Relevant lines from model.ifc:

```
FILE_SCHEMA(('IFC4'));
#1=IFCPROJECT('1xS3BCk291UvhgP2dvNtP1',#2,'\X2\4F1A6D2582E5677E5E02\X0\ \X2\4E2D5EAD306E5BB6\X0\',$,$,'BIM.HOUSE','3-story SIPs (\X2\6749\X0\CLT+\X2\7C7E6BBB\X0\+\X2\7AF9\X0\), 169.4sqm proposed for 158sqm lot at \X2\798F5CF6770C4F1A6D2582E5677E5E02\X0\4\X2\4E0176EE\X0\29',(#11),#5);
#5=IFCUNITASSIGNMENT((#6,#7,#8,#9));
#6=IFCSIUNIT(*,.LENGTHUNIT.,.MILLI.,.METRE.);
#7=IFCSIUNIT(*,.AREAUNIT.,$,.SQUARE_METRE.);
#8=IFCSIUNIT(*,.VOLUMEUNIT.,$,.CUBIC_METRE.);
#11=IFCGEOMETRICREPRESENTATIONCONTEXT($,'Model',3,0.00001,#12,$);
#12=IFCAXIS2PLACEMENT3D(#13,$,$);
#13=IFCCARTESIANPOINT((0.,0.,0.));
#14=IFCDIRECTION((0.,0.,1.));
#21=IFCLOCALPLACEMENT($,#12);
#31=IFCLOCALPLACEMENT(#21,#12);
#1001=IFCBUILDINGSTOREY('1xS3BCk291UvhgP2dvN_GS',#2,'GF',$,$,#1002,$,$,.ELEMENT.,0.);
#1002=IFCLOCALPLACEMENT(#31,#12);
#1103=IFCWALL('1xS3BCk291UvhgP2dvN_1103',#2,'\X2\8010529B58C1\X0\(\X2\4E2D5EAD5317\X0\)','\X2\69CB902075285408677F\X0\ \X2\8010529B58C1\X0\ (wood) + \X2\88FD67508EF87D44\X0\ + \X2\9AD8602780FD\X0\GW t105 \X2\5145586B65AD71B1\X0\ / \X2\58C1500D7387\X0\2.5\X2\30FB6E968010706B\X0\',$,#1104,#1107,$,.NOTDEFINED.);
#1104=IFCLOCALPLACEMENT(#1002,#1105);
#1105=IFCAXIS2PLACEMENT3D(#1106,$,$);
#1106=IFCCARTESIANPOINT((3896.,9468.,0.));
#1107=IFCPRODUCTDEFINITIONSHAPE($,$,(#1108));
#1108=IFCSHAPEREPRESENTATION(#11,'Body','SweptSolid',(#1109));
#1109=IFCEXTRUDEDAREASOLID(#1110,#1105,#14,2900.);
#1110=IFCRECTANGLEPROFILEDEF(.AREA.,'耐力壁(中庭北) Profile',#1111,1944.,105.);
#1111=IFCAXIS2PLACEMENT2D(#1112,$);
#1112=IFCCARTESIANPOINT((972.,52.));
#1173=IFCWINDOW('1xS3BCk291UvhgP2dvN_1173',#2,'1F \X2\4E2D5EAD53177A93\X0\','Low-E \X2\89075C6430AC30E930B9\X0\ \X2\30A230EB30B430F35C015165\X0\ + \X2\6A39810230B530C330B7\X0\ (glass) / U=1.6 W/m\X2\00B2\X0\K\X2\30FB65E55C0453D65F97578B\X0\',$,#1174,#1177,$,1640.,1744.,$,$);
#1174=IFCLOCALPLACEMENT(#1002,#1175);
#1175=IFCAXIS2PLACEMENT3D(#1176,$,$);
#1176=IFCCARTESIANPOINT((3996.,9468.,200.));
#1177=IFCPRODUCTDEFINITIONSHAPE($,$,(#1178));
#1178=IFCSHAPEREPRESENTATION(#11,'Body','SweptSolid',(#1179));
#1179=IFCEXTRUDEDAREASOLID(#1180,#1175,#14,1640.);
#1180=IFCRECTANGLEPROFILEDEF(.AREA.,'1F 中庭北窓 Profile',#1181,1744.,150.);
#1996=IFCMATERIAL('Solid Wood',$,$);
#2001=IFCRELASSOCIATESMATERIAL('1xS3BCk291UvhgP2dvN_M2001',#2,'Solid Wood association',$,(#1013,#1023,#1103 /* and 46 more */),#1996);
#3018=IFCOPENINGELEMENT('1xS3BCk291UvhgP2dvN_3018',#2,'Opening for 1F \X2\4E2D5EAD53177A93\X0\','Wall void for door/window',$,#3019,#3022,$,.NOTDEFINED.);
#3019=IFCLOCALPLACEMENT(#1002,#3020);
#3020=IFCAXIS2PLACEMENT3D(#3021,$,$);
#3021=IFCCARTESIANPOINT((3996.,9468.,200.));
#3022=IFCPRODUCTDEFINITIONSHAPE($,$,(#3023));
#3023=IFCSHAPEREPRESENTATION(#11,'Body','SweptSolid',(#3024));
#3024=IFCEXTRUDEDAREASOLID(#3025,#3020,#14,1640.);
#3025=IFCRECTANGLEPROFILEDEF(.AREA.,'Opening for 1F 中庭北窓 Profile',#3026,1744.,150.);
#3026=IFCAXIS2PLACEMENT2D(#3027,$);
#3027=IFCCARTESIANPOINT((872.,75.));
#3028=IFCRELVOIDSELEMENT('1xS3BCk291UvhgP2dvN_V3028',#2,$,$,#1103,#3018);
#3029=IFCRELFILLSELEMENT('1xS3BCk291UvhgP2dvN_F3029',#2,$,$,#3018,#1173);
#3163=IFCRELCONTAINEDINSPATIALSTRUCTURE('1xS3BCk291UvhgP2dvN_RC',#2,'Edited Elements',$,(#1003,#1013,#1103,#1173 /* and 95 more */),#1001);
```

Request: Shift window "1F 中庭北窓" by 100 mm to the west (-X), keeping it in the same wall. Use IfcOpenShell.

```python
import ifcopenshell
import ifcopenshell.api.geometry
import ifcopenshell.util.placement

model = ifcopenshell.open("model.ifc")

window = model.by_guid("1xS3BCk291UvhgP2dvN_1173")
opening = window.FillsVoids[0].RelatingOpeningElement
wall = opening.VoidsElements[0].RelatingBuildingElement

wall_matrix = ifcopenshell.util.placement.get_local_placement(wall.ObjectPlacement)
shift = wall_matrix[:3, 0] * -100.0
before = ifcopenshell.util.placement.get_local_placement(window.ObjectPlacement)[:3, 3].copy()

# The window is not placed relative to its opening, so move both.
for product in (opening, window):
    matrix = ifcopenshell.util.placement.get_local_placement(product.ObjectPlacement)
    matrix[:3, 3] += shift
    ifcopenshell.api.geometry.edit_object_placement(model, product=product, matrix=matrix, is_si=False)

after = ifcopenshell.util.placement.get_local_placement(window.ObjectPlacement)[:3, 3]
print("window moved by", (after - before).round(3) + 0.0)

model.write("model_edited.ifc")
```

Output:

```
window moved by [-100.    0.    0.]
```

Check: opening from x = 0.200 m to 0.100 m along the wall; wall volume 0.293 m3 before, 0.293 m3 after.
